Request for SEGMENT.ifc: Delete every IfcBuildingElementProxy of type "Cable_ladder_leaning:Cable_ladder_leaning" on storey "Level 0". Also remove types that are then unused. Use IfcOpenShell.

First a look at what the model holds.

```python
import ifcopenshell
import ifcopenshell.util.element

model = ifcopenshell.open("SEGMENT.ifc")
print(model.schema)
storey = next(s for s in model.by_type("IfcBuildingStorey") if s.Name == "Level 0")
proxies = [e for e in ifcopenshell.util.element.get_decomposition(storey) if e.is_a("IfcBuildingElementProxy")]
seen = {}
for e in proxies:
    element_type = ifcopenshell.util.element.get_type(e)
    name = element_type.Name if element_type not in (None, e) else None
    seen[name] = seen.get(name, 0) + 1
for name, count in sorted(seen.items(), key=str):
    print(count, "x", name)
```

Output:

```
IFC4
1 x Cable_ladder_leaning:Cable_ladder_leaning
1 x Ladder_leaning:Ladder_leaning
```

```python
import ifcopenshell
import ifcopenshell.api.root
import ifcopenshell.util.element

model = ifcopenshell.open("SEGMENT.ifc")

storey = next(s for s in model.by_type("IfcBuildingStorey") if s.Name == "Level 0")
proxies = [e for e in ifcopenshell.util.element.get_decomposition(storey) if e.is_a("IfcBuildingElementProxy")]
targets = [e for e in proxies if (t := ifcopenshell.util.element.get_type(e)) not in (None, e) and t.Name == "Cable_ladder_leaning:Cable_ladder_leaning"]
types = {ifcopenshell.util.element.get_type(e) for e in targets} - {None, *targets}

for e in targets:
    ifcopenshell.api.root.remove_product(model, product=e)
print(len(targets), "removed")

unused = [t for t in types if not ifcopenshell.util.element.get_types(t)]
for t in unused:
    ifcopenshell.api.root.remove_product(model, product=t)
print(len(unused), "unused types removed")

model.write("SEGMENT_v2.ifc")
```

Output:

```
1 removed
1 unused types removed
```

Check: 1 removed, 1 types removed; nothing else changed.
